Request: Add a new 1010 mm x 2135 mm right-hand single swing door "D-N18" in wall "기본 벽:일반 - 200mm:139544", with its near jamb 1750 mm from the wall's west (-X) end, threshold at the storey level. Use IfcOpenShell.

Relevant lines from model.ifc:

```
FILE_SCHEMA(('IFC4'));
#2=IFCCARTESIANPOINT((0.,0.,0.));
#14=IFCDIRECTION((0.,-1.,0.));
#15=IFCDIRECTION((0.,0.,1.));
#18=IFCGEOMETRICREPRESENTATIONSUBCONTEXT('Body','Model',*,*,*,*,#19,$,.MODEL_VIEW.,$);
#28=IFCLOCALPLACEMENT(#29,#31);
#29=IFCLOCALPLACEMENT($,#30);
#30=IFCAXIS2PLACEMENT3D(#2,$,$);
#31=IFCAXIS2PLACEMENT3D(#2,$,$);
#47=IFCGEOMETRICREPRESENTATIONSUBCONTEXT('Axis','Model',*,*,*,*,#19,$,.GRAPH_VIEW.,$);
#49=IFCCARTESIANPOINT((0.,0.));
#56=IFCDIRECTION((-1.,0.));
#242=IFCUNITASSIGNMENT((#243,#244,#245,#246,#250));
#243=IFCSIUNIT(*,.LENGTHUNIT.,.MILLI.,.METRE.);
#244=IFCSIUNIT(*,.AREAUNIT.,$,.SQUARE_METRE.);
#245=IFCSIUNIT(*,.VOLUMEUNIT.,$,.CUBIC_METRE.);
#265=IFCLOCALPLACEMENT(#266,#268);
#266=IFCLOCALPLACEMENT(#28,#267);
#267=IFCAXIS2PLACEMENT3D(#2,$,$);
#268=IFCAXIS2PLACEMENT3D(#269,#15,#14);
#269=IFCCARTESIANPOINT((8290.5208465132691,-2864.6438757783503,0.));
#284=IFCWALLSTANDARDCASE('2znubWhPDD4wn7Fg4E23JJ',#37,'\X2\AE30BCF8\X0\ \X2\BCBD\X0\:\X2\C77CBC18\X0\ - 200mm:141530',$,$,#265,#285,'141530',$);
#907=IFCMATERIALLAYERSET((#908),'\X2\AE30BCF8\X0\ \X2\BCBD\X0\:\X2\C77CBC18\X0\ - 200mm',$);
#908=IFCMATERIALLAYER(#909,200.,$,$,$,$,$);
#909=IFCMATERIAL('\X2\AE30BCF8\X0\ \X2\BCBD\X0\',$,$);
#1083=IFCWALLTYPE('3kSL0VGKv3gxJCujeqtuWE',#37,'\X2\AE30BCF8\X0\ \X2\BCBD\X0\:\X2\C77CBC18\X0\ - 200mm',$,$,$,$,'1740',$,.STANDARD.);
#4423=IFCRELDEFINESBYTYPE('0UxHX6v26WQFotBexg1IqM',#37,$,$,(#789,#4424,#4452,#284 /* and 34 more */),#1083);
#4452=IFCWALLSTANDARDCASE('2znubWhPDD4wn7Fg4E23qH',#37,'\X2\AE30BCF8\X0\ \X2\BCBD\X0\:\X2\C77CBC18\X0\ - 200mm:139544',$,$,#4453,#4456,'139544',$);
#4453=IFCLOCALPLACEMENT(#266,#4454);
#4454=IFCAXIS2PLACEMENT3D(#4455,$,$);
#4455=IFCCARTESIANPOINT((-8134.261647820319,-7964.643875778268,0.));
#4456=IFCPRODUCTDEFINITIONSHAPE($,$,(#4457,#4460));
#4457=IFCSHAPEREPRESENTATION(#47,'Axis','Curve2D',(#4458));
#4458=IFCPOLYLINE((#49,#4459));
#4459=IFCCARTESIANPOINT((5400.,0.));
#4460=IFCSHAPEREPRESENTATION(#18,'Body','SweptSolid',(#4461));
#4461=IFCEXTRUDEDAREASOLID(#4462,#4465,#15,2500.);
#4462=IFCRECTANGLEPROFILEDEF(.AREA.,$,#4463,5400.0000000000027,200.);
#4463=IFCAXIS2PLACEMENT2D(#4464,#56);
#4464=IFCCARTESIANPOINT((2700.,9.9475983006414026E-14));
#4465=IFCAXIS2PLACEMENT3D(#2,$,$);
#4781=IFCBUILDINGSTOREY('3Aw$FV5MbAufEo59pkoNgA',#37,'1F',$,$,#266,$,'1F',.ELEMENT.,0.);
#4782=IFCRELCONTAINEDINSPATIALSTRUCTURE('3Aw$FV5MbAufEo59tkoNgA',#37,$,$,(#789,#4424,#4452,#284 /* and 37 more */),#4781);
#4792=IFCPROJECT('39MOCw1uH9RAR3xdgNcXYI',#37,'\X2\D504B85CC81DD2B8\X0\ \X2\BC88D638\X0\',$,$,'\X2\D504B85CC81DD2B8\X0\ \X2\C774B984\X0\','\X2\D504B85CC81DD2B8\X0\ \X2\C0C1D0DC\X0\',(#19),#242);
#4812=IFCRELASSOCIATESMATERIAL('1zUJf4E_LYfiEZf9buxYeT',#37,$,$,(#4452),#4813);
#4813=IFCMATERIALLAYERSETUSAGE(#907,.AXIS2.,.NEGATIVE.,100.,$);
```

```python
import numpy as np
import ifcopenshell
import ifcopenshell.api.feature
import ifcopenshell.api.geometry
import ifcopenshell.api.root
import ifcopenshell.api.spatial
import ifcopenshell.geom
import ifcopenshell.util.element
import ifcopenshell.util.placement
import ifcopenshell.util.representation
import ifcopenshell.util.shape
import ifcopenshell.util.unit

model = ifcopenshell.open("model.ifc")
unit_scale = ifcopenshell.util.unit.calculate_unit_scale(model)
settings = ifcopenshell.geom.settings()


def volume(element):
    """Net volume in cubic metres, openings subtracted."""
    shape = ifcopenshell.geom.create_shape(settings, element)
    return ifcopenshell.util.shape.get_volume(shape.geometry)


wall = model.by_guid("2znubWhPDD4wn7Fg4E23qH")
storey = ifcopenshell.util.element.get_container(wall, ifc_class="IfcBuildingStorey")
context = ifcopenshell.util.representation.get_context(model, "Model", "Body", "MODEL_VIEW")
before = volume(wall)

width, height, from_end, sill = 1.01, 2.135, 1.75, 0.0  # metres

# The wall runs along its own X axis, and the end named is its -X end.
wall_shape = ifcopenshell.geom.create_shape(settings, wall)
x, y, z = ifcopenshell.util.shape.get_vertices(wall_shape.geometry).T
start = x.min() + from_end
face, thickness = float(y.min()), float(y.max() - y.min())
wall_matrix = ifcopenshell.util.placement.get_local_placement(wall.ObjectPlacement)
level = ifcopenshell.util.placement.get_local_placement(storey.ObjectPlacement)[2, 3]


def in_wall(x, y):
    """Placement at x, y metres in the wall's axes, at sill height."""
    matrix = wall_matrix.copy()
    matrix[:, 3] = wall_matrix @ np.array([x / unit_scale, y / unit_scale, 0.0, 1.0])
    matrix[2, 3] = level + sill / unit_scale
    return matrix


# Opening: a box that overshoots both wall faces by 50 mm.
opening = ifcopenshell.api.root.create_entity(model, ifc_class="IfcOpeningElement", predefined_type="OPENING")
box = ifcopenshell.api.geometry.add_wall_representation(
    model, context=context, length=width, height=height, thickness=thickness + 0.1
)
ifcopenshell.api.geometry.assign_representation(model, product=opening, representation=box)
ifcopenshell.api.geometry.edit_object_placement(model, product=opening, matrix=in_wall(start, face - 0.05), is_si=False)
ifcopenshell.api.feature.add_feature(model, feature=opening, element=wall)

door = ifcopenshell.api.root.create_entity(model, ifc_class="IfcDoor", name="D-N18", predefined_type="DOOR")
door.OverallWidth, door.OverallHeight = width / unit_scale, height / unit_scale
door.OperationType = "SINGLE_SWING_RIGHT"
body = ifcopenshell.api.geometry.add_door_representation(
    model,
    context=context,
    overall_width=door.OverallWidth,
    overall_height=door.OverallHeight,
    operation_type="SINGLE_SWING_RIGHT",
    lining_properties={"LiningDepth": thickness / unit_scale, "ThresholdDepth": thickness / unit_scale},
)
ifcopenshell.api.geometry.assign_representation(model, product=door, representation=body)
ifcopenshell.api.spatial.assign_container(model, products=[door], relating_structure=storey)
ifcopenshell.api.feature.add_filling(model, opening=opening, element=door)

# The lining spans the wall, so the door starts at the wall face.
ifcopenshell.api.geometry.edit_object_placement(model, product=door, matrix=in_wall(start, face), is_si=False)

after = volume(wall)

print(f"wall volume {before:.3f} -> {after:.3f} m3")

model.write("model_updated.ifc")
```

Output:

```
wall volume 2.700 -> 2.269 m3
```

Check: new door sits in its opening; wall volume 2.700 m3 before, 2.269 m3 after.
